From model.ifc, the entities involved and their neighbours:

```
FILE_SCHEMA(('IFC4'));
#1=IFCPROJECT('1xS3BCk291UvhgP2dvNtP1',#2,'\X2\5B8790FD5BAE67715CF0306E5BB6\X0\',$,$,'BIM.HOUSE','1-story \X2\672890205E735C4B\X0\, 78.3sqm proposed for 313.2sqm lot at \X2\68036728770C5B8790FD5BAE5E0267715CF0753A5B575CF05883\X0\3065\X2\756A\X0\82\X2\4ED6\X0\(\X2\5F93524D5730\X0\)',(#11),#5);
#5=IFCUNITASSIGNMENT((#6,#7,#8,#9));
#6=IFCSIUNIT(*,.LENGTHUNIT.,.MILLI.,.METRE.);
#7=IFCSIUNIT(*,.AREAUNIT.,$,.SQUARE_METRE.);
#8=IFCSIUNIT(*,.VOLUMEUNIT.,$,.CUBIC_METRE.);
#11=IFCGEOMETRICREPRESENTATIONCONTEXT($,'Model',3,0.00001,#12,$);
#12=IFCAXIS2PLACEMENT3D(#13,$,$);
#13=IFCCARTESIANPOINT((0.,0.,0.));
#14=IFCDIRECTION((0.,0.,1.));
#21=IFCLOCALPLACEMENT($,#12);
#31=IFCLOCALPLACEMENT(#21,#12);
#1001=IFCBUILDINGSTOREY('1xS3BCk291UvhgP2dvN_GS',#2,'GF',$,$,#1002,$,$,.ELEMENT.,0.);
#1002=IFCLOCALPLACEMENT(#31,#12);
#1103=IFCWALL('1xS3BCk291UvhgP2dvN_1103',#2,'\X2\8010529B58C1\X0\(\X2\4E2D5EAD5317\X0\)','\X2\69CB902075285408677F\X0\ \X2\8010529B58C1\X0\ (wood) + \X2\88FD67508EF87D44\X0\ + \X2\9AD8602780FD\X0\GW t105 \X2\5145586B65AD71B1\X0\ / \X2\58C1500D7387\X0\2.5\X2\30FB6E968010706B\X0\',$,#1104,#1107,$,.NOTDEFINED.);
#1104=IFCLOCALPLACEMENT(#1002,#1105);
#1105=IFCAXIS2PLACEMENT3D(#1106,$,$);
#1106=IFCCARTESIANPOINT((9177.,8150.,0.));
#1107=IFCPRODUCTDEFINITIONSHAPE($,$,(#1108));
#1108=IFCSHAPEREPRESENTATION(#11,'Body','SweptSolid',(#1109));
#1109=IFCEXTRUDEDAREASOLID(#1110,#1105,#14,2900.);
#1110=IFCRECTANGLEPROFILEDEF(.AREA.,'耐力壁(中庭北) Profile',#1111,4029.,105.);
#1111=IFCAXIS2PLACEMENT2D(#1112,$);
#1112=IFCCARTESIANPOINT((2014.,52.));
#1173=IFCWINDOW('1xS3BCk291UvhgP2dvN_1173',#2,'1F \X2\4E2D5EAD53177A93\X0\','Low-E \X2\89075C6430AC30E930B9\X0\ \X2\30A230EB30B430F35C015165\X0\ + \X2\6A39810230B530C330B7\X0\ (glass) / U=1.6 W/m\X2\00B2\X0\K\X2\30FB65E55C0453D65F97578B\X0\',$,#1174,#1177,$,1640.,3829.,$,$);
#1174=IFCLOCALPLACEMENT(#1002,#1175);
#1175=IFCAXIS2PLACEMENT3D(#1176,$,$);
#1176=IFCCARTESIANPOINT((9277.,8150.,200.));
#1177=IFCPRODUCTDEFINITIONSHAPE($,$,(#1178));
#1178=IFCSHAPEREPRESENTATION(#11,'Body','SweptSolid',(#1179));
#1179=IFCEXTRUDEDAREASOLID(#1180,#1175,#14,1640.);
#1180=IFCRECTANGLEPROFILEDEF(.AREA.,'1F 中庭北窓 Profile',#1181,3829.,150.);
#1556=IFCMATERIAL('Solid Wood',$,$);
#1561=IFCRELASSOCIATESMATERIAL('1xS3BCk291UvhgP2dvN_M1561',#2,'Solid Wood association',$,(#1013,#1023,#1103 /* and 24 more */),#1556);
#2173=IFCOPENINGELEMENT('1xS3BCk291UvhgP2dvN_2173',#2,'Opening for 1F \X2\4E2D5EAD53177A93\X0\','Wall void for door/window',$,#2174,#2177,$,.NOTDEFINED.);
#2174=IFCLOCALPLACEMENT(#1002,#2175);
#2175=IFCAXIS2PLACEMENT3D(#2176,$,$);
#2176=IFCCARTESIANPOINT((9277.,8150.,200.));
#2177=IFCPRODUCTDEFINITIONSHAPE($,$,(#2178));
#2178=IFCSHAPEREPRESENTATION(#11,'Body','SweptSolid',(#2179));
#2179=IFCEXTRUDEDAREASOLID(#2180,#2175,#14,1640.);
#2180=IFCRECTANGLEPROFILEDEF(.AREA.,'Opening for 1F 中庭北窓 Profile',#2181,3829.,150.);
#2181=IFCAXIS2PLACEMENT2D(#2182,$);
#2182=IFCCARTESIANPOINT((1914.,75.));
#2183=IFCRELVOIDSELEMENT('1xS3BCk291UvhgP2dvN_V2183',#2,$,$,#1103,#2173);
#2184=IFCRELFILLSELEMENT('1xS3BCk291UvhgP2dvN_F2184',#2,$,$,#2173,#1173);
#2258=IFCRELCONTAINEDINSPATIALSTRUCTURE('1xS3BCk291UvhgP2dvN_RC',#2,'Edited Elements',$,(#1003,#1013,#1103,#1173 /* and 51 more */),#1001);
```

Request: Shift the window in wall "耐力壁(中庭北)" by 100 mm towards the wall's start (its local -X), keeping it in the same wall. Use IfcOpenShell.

```python
import ifcopenshell
import ifcopenshell.api.geometry
import ifcopenshell.util.placement
import ifcopenshell.util.unit

model = ifcopenshell.open("model.ifc")
unit_scale = ifcopenshell.util.unit.calculate_unit_scale(model)

window = model.by_guid("1xS3BCk291UvhgP2dvN_1173")
opening = window.FillsVoids[0].RelatingOpeningElement
wall = opening.VoidsElements[0].RelatingBuildingElement

wall_matrix = ifcopenshell.util.placement.get_local_placement(wall.ObjectPlacement)
shift = wall_matrix[:3, 0] * -0.1 / unit_scale
before = ifcopenshell.util.placement.get_local_placement(window.ObjectPlacement)[:3, 3].copy()

# The window is not placed relative to its opening, so move both.
for product in (opening, window):
    matrix = ifcopenshell.util.placement.get_local_placement(product.ObjectPlacement)
    matrix[:3, 3] += shift
    ifcopenshell.api.geometry.edit_object_placement(model, product=product, matrix=matrix, is_si=False)

after = ifcopenshell.util.placement.get_local_placement(window.ObjectPlacement)[:3, 3]
print("window moved by", (after - before).round(3) + 0.0)

model.write("model-out.ifc")
```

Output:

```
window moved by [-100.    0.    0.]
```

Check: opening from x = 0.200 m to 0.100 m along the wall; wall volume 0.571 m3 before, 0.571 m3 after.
